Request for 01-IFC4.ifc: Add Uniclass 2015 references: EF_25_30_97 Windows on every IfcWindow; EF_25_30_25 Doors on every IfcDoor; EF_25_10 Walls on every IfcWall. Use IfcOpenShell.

First a look at what the model holds.

```python
import ifcopenshell

model = ifcopenshell.open("01-IFC4.ifc")
print(model.schema)
print("classifications:", [c.Name for c in model.by_type("IfcClassification")])
for ifc_class in ("IfcDoor", "IfcRoof", "IfcStair", "IfcWall", "IfcWindow"):
    print(ifc_class, len(model.by_type(ifc_class)))
```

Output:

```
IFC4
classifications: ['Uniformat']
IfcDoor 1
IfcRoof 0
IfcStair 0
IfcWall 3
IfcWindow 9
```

```python
import ifcopenshell
import ifcopenshell.api.classification

model = ifcopenshell.open("01-IFC4.ifc")

system = ifcopenshell.api.classification.add_classification(model, classification="Uniclass 2015")

codes = {
    "IfcWindow": ("EF_25_30_97", "Windows"),
    "IfcDoor": ("EF_25_30_25", "Doors"),
    "IfcWall": ("EF_25_10", "Walls"),
}
for ifc_class, (code, name) in codes.items():
    products = model.by_type(ifc_class)
    ifcopenshell.api.classification.add_reference(
        model, products=products, classification=system, identification=code, name=name
    )
    print(code, len(products))

model.write("01-IFC4_rev.ifc")
```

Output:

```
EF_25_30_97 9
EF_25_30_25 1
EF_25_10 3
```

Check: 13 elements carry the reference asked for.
